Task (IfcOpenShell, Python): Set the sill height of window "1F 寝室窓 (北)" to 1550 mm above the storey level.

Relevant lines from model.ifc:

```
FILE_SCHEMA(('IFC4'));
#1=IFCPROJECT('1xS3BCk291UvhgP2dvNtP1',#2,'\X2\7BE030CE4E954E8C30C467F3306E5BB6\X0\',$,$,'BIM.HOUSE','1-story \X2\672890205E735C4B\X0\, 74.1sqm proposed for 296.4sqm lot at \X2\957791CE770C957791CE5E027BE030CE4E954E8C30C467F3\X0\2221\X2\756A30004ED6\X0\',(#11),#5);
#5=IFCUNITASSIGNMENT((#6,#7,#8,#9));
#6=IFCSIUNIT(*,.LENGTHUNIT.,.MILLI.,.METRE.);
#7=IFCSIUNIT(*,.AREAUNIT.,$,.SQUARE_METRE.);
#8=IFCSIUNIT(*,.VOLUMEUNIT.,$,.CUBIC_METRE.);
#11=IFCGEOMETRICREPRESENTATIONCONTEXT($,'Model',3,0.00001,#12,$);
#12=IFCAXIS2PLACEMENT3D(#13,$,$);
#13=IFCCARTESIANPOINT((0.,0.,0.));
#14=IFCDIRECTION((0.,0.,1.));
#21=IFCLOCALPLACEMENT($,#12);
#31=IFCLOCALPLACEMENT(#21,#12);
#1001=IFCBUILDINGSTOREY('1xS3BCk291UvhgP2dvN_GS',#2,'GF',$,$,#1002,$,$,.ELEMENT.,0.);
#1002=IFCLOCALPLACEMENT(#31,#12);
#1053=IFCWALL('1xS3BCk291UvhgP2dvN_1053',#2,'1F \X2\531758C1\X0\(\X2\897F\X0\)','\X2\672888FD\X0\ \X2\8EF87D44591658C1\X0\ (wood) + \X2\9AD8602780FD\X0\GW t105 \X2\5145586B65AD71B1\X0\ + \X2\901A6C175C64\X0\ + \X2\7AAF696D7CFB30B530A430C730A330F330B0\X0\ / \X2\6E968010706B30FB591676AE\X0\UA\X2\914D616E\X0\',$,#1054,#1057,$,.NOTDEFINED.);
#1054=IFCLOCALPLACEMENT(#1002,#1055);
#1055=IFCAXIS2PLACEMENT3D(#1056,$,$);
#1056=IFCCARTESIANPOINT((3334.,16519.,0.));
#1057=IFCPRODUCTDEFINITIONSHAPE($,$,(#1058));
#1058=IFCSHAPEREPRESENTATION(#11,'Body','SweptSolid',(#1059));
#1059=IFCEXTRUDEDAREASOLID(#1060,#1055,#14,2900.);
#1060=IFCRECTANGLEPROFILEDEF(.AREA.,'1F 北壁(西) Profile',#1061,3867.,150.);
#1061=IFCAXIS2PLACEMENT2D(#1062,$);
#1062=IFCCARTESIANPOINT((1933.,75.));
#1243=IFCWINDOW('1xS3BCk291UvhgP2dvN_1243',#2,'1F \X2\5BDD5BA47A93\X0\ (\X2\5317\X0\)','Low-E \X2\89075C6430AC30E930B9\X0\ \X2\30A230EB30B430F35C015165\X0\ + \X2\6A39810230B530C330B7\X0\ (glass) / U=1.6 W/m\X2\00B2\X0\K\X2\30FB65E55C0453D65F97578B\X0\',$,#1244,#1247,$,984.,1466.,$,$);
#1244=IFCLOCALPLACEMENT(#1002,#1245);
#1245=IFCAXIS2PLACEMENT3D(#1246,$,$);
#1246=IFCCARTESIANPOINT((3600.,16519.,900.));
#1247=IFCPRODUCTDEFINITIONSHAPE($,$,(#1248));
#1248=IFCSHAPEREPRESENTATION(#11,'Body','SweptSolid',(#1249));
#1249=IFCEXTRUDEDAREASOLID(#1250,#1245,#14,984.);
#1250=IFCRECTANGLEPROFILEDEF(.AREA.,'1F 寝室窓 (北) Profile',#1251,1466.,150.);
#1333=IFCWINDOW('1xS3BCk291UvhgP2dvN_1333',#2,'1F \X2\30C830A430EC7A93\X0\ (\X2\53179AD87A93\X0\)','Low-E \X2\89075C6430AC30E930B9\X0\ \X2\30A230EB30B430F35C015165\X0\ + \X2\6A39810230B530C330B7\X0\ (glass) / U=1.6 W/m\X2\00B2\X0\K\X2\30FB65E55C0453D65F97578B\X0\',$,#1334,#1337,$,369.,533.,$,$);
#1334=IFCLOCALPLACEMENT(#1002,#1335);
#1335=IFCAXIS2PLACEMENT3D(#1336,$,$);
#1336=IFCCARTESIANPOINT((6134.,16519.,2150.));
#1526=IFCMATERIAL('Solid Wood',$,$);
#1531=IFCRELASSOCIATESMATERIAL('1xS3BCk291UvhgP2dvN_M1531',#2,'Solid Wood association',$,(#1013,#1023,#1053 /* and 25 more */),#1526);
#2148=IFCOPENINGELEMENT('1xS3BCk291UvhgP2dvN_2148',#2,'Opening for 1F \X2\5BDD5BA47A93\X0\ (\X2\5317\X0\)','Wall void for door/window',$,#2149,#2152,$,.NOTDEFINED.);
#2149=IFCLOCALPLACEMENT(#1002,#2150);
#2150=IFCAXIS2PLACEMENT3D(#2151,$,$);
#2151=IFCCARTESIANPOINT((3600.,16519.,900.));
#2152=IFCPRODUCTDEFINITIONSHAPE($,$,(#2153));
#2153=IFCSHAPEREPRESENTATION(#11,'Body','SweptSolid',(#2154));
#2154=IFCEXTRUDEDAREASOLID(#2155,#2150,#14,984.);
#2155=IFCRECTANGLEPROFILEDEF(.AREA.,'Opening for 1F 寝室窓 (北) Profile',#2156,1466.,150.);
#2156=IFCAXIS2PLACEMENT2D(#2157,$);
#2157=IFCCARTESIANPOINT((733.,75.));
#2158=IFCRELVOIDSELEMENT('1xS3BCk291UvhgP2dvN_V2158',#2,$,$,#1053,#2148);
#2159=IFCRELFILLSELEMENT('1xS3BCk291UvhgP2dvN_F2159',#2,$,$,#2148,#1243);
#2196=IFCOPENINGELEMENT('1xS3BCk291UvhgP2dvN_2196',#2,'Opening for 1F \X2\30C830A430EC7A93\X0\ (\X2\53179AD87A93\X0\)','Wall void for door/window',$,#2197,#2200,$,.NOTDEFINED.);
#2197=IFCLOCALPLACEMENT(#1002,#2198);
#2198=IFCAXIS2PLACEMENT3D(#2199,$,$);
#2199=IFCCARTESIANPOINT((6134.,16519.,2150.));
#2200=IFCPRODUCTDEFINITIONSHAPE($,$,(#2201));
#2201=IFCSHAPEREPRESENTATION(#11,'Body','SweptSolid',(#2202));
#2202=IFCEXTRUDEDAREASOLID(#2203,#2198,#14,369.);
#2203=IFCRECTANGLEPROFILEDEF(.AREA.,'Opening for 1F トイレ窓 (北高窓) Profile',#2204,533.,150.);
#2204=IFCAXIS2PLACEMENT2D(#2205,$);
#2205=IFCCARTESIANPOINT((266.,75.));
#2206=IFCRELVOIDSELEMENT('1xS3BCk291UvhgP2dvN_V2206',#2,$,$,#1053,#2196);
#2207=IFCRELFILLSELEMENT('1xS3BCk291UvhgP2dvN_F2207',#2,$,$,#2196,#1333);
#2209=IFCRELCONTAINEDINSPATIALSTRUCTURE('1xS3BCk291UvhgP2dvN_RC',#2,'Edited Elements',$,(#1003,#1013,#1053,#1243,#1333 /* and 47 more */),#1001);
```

```python
import numpy as np
import ifcopenshell
import ifcopenshell.api.geometry
import ifcopenshell.geom
import ifcopenshell.util.element
import ifcopenshell.util.placement
import ifcopenshell.util.shape
import ifcopenshell.util.unit

model = ifcopenshell.open("model.ifc")
unit_scale = ifcopenshell.util.unit.calculate_unit_scale(model)

window = model.by_guid("1xS3BCk291UvhgP2dvN_1243")
opening = window.FillsVoids[0].RelatingOpeningElement
storey = ifcopenshell.util.element.get_container(window, ifc_class="IfcBuildingStorey")
level = ifcopenshell.util.placement.get_local_placement(storey.ObjectPlacement)[2, 3]

# The opening's origin need not be at the sill, so measure its lowest point.
shape = ifcopenshell.geom.create_shape(ifcopenshell.geom.settings(), opening)
bottom = ifcopenshell.util.shape.get_shape_bottom_elevation(shape, shape.geometry) / unit_scale
dz = level + 1.55 / unit_scale - bottom

shift = np.array([0.0, 0.0, dz])
# The window is not placed relative to its opening, so move both.
for product in (opening, window):
    matrix = ifcopenshell.util.placement.get_local_placement(product.ObjectPlacement)
    matrix[:3, 3] += shift
    ifcopenshell.api.geometry.edit_object_placement(model, product=product, matrix=matrix, is_si=False)

print(f"moved by {dz * unit_scale:+.3f} m")

model.write("model_edited.ifc")
```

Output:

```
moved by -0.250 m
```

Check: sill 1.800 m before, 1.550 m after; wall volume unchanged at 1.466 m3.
